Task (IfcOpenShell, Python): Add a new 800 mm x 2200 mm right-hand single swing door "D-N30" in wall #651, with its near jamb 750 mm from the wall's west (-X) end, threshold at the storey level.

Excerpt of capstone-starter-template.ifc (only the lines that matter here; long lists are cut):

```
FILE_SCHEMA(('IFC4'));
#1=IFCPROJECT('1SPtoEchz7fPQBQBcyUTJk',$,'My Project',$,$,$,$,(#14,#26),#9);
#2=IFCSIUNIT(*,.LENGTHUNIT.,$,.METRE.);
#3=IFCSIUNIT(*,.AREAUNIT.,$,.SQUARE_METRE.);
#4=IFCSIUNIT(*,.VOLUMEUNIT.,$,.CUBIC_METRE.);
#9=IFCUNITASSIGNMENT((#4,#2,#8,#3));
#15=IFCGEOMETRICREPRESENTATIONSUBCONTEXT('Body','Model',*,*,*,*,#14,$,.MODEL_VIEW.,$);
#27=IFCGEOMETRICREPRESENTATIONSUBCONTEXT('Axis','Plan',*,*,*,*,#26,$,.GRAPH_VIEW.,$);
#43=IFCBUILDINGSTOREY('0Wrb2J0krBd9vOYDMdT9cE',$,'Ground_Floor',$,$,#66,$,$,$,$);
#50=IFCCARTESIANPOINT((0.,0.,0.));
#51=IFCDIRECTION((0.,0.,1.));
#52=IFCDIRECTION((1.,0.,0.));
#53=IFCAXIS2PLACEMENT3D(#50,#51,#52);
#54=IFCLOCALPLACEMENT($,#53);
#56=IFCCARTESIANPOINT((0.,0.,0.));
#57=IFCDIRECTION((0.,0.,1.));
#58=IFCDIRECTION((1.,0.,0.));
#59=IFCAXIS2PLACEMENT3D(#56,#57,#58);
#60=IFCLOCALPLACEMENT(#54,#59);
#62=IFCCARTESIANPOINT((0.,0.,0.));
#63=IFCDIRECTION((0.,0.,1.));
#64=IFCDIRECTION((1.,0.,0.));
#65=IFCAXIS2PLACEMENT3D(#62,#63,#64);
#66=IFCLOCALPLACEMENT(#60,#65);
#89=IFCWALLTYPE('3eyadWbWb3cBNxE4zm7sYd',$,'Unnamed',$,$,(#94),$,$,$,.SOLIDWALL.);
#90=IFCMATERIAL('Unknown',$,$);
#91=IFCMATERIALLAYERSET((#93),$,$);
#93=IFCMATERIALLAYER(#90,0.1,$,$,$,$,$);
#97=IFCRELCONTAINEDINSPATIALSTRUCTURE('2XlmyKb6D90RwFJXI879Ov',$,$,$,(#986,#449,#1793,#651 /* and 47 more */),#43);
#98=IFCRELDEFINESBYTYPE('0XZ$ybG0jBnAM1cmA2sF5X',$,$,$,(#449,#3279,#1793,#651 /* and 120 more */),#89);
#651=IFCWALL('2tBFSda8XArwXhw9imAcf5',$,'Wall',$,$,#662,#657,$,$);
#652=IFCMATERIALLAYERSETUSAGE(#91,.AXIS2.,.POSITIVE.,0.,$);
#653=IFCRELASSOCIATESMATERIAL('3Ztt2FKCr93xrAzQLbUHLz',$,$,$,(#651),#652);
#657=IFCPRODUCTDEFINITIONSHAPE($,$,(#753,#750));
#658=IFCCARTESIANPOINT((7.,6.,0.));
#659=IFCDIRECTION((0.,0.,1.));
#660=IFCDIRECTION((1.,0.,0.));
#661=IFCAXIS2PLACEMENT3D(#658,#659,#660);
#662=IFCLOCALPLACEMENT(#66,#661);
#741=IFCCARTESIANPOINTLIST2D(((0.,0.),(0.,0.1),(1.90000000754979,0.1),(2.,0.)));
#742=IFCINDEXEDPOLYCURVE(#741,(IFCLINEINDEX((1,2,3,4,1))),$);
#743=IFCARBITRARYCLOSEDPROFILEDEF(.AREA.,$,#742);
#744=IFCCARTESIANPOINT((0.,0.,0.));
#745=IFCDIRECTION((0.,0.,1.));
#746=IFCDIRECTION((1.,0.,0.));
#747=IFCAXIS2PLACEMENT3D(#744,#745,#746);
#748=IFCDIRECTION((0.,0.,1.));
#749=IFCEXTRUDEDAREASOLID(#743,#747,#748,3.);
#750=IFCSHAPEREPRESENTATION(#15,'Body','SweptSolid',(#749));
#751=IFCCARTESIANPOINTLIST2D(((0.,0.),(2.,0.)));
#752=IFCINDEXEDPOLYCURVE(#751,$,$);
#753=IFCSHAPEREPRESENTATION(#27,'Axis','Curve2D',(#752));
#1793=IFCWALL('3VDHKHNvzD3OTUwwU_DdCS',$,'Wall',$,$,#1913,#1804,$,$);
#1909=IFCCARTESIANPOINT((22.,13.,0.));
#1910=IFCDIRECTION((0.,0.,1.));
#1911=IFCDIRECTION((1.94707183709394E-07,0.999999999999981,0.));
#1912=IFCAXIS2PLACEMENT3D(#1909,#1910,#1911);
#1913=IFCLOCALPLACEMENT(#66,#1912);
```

```python
import numpy as np
import ifcopenshell
import ifcopenshell.api.feature
import ifcopenshell.api.geometry
import ifcopenshell.api.root
import ifcopenshell.api.spatial
import ifcopenshell.geom
import ifcopenshell.util.element
import ifcopenshell.util.placement
import ifcopenshell.util.representation
import ifcopenshell.util.shape
import ifcopenshell.util.unit

model = ifcopenshell.open("capstone-starter-template.ifc")
unit_scale = ifcopenshell.util.unit.calculate_unit_scale(model)
settings = ifcopenshell.geom.settings()


def volume(element):
    """Net volume in cubic metres, openings subtracted."""
    shape = ifcopenshell.geom.create_shape(settings, element)
    return ifcopenshell.util.shape.get_volume(shape.geometry)


wall = model.by_guid("2tBFSda8XArwXhw9imAcf5")
storey = ifcopenshell.util.element.get_container(wall, ifc_class="IfcBuildingStorey")
context = ifcopenshell.util.representation.get_context(model, "Model", "Body", "MODEL_VIEW")
before = volume(wall)

width, height, from_end, sill = 0.8, 2.2, 0.75, 0.0  # metres

# The wall runs along its own X axis, and the end named is its -X end.
wall_shape = ifcopenshell.geom.create_shape(settings, wall)
x, y, z = ifcopenshell.util.shape.get_vertices(wall_shape.geometry).T
start = x.min() + from_end
face, thickness = float(y.min()), float(y.max() - y.min())
wall_matrix = ifcopenshell.util.placement.get_local_placement(wall.ObjectPlacement)
level = ifcopenshell.util.placement.get_local_placement(storey.ObjectPlacement)[2, 3]


def in_wall(x, y):
    """Placement at x, y metres in the wall's axes, at sill height."""
    matrix = wall_matrix.copy()
    matrix[:, 3] = wall_matrix @ np.array([x / unit_scale, y / unit_scale, 0.0, 1.0])
    matrix[2, 3] = level + sill / unit_scale
    return matrix


# Opening: a box that overshoots both wall faces by 50 mm.
opening = ifcopenshell.api.root.create_entity(model, ifc_class="IfcOpeningElement", predefined_type="OPENING")
box = ifcopenshell.api.geometry.add_wall_representation(
    model, context=context, length=width, height=height, thickness=thickness + 0.1
)
ifcopenshell.api.geometry.assign_representation(model, product=opening, representation=box)
ifcopenshell.api.geometry.edit_object_placement(model, product=opening, matrix=in_wall(start, face - 0.05), is_si=False)
ifcopenshell.api.feature.add_feature(model, feature=opening, element=wall)

door = ifcopenshell.api.root.create_entity(model, ifc_class="IfcDoor", name="D-N30", predefined_type="DOOR")
door.OverallWidth, door.OverallHeight = width / unit_scale, height / unit_scale
door.OperationType = "SINGLE_SWING_RIGHT"
body = ifcopenshell.api.geometry.add_door_representation(
    model,
    context=context,
    overall_width=door.OverallWidth,
    overall_height=door.OverallHeight,
    operation_type="SINGLE_SWING_RIGHT",
    lining_properties={"LiningDepth": thickness / unit_scale, "ThresholdDepth": thickness / unit_scale},
)
ifcopenshell.api.geometry.assign_representation(model, product=door, representation=body)
ifcopenshell.api.spatial.assign_container(model, products=[door], relating_structure=storey)
ifcopenshell.api.feature.add_filling(model, opening=opening, element=door)

# The lining spans the wall, so the door starts at the wall face.
ifcopenshell.api.geometry.edit_object_placement(model, product=door, matrix=in_wall(start, face), is_si=False)

after = volume(wall)

print(f"wall volume {before:.3f} -> {after:.3f} m3")

model.write("capstone-starter-template_updated.ifc")
```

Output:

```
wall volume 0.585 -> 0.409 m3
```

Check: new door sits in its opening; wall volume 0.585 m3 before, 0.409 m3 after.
